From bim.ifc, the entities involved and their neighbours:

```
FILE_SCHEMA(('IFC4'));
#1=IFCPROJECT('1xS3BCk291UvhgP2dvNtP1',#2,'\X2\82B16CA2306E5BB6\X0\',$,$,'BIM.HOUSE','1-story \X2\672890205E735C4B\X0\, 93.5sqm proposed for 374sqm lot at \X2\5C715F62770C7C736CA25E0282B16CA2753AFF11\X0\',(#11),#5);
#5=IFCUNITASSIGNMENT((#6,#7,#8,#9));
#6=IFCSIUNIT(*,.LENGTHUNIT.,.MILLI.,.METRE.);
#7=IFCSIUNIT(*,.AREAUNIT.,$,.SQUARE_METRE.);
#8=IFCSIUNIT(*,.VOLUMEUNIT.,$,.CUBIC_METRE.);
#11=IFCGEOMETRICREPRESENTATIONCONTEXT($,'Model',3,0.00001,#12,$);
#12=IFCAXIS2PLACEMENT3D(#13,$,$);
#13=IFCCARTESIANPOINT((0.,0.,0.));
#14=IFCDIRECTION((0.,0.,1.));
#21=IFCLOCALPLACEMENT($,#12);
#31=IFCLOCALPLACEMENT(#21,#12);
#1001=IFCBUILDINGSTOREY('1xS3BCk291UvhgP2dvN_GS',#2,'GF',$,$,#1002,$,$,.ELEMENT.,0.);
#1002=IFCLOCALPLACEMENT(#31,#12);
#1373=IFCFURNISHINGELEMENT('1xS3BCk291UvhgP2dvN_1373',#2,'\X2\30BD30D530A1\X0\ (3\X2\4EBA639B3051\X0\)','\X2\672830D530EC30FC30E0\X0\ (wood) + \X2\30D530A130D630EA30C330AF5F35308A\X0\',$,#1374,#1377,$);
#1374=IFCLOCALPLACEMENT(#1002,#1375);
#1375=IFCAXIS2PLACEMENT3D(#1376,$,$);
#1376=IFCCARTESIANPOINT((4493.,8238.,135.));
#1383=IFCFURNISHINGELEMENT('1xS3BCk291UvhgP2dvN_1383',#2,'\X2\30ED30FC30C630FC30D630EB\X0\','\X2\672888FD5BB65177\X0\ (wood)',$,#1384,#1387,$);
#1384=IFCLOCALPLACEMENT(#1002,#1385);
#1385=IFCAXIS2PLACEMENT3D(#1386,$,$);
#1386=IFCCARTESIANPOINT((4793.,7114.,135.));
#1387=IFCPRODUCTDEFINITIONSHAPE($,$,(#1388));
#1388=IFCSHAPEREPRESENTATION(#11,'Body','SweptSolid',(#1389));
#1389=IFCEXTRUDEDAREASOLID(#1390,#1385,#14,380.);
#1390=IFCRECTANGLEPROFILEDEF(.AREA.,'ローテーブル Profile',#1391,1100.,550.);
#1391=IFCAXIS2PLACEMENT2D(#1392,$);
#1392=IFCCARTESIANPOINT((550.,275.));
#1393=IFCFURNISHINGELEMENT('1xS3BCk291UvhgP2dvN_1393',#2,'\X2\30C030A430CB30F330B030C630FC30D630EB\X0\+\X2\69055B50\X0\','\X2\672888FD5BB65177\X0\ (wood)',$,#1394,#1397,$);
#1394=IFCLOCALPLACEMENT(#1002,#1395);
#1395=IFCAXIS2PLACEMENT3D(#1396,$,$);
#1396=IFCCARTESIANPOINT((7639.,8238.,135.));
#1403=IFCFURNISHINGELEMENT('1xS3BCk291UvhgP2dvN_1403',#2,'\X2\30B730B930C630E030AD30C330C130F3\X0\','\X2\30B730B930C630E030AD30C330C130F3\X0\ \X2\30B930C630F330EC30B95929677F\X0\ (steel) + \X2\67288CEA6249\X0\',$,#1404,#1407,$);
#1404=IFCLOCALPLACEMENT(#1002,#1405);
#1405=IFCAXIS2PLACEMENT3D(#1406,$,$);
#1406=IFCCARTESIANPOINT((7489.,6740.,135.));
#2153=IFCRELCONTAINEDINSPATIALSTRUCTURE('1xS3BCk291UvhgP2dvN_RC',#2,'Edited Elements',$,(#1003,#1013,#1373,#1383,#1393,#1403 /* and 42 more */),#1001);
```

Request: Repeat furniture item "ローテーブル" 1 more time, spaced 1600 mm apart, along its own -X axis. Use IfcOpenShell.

```python
import ifcopenshell
import ifcopenshell.api.geometry
import ifcopenshell.api.root
import ifcopenshell.util.element
import ifcopenshell.util.placement

model = ifcopenshell.open("bim.ifc")


def reuse_history(source, copy):
    """copy_class also copies each property set's owner history, people and application; keep the originals."""
    for rel in copy.IsDefinedBy:
        if rel.is_a("IfcRelDefinesByProperties") and (history := rel.RelatingPropertyDefinition.OwnerHistory):
            rel.RelatingPropertyDefinition.OwnerHistory = source.OwnerHistory
            ifcopenshell.util.element.remove_deep2(model, history)


source = model.by_guid("1xS3BCk291UvhgP2dvN_1383")
base = ifcopenshell.util.placement.get_local_placement(source.ObjectPlacement)
step = -base[:3, 0] * 1600.0

for i in range(1, 2):
    copy = ifcopenshell.api.root.copy_class(model, product=source)
    copy.Representation = ifcopenshell.util.element.copy_deep(
        model, source.Representation, exclude=["IfcGeometricRepresentationContext", "IfcRepresentationMap"]
    )
    reuse_history(source, copy)
    matrix = base.copy()
    matrix[:3, 3] += i * step
    print("added at", matrix[:3, 3].round(3) + 0.0)
    ifcopenshell.api.geometry.edit_object_placement(model, product=copy, matrix=matrix, is_si=False)

model.write("bim_edited.ifc")
```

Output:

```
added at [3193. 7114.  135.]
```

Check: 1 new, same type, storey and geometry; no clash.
